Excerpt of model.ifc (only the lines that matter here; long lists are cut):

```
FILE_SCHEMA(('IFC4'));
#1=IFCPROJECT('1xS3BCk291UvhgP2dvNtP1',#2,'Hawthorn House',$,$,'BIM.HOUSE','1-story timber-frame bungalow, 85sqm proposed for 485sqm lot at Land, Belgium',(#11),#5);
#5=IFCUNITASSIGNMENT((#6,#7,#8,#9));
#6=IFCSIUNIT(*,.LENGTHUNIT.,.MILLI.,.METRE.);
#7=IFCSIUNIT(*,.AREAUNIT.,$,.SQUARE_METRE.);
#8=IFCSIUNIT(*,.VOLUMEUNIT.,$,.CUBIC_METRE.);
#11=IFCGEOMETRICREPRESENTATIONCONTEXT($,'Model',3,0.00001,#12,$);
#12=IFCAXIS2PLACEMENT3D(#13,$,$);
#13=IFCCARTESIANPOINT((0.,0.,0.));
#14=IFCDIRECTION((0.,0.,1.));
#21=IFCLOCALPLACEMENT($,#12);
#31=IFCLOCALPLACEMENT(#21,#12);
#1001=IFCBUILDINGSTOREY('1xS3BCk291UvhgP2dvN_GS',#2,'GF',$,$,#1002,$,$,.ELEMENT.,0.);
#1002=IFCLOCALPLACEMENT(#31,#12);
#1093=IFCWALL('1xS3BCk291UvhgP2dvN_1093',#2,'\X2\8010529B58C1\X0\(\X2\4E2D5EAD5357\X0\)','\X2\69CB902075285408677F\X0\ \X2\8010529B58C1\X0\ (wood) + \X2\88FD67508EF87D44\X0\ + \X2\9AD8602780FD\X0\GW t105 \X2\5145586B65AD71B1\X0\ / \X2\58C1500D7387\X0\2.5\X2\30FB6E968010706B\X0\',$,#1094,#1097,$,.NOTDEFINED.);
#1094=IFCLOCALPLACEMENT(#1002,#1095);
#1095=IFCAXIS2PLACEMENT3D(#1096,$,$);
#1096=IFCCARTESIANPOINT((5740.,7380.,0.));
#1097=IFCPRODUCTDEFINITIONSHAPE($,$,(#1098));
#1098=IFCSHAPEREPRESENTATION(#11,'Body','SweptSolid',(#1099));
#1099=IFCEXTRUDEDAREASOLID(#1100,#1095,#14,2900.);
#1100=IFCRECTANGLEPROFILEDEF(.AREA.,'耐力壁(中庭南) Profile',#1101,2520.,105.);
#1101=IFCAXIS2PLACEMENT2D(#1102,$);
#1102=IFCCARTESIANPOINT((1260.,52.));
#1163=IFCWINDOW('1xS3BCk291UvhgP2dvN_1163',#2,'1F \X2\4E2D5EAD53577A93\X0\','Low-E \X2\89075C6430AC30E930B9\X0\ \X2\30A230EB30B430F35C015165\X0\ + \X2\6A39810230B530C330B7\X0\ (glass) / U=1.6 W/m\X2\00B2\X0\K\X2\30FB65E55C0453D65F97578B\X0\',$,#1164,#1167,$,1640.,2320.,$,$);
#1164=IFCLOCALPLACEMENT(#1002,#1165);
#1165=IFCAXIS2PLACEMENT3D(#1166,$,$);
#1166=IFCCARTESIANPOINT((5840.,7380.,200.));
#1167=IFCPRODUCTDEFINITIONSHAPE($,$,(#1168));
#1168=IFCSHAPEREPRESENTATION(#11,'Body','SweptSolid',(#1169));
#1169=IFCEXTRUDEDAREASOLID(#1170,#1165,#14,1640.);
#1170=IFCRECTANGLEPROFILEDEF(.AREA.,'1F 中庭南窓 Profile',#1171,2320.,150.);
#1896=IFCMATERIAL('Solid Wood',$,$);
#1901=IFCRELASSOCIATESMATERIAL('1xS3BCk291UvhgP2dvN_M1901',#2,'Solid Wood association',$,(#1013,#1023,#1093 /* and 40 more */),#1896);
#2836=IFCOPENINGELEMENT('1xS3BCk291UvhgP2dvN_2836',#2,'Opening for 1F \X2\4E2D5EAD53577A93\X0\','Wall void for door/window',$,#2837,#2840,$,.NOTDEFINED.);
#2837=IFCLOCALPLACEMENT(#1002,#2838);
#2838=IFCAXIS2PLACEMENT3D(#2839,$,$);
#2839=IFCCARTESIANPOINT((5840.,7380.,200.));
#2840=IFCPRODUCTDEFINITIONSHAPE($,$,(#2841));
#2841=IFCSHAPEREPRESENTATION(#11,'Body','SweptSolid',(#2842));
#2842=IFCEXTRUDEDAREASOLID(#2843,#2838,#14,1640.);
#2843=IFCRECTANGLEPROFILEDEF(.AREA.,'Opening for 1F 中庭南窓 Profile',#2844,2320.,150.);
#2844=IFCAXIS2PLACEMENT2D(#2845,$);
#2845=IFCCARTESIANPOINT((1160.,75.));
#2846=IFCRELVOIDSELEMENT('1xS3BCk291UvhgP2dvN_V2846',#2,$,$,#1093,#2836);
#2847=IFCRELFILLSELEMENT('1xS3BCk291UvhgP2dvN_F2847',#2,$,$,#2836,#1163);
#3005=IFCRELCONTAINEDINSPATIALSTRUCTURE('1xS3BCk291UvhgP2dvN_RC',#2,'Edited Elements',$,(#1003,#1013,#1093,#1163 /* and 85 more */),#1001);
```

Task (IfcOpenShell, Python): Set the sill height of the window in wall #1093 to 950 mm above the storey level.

```python
import numpy as np
import ifcopenshell
import ifcopenshell.api.geometry
import ifcopenshell.geom
import ifcopenshell.util.element
import ifcopenshell.util.placement
import ifcopenshell.util.shape
import ifcopenshell.util.unit

model = ifcopenshell.open("model.ifc")
unit_scale = ifcopenshell.util.unit.calculate_unit_scale(model)

window = model.by_id(1163)
opening = window.FillsVoids[0].RelatingOpeningElement
storey = ifcopenshell.util.element.get_container(window, ifc_class="IfcBuildingStorey")
level = ifcopenshell.util.placement.get_local_placement(storey.ObjectPlacement)[2, 3]

# The opening's origin need not be at the sill, so measure its lowest point.
shape = ifcopenshell.geom.create_shape(ifcopenshell.geom.settings(), opening)
bottom = ifcopenshell.util.shape.get_shape_bottom_elevation(shape, shape.geometry) / unit_scale
dz = level + 0.95 / unit_scale - bottom

shift = np.array([0.0, 0.0, dz])
# The window is not placed relative to its opening, so move both.
for product in (opening, window):
    matrix = ifcopenshell.util.placement.get_local_placement(product.ObjectPlacement)
    matrix[:3, 3] += shift
    ifcopenshell.api.geometry.edit_object_placement(model, product=product, matrix=matrix, is_si=False)

print(f"moved by {dz * unit_scale:+.3f} m")

model.write("model_rev.ifc")
```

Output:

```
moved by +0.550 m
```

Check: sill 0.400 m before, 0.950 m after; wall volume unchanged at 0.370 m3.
